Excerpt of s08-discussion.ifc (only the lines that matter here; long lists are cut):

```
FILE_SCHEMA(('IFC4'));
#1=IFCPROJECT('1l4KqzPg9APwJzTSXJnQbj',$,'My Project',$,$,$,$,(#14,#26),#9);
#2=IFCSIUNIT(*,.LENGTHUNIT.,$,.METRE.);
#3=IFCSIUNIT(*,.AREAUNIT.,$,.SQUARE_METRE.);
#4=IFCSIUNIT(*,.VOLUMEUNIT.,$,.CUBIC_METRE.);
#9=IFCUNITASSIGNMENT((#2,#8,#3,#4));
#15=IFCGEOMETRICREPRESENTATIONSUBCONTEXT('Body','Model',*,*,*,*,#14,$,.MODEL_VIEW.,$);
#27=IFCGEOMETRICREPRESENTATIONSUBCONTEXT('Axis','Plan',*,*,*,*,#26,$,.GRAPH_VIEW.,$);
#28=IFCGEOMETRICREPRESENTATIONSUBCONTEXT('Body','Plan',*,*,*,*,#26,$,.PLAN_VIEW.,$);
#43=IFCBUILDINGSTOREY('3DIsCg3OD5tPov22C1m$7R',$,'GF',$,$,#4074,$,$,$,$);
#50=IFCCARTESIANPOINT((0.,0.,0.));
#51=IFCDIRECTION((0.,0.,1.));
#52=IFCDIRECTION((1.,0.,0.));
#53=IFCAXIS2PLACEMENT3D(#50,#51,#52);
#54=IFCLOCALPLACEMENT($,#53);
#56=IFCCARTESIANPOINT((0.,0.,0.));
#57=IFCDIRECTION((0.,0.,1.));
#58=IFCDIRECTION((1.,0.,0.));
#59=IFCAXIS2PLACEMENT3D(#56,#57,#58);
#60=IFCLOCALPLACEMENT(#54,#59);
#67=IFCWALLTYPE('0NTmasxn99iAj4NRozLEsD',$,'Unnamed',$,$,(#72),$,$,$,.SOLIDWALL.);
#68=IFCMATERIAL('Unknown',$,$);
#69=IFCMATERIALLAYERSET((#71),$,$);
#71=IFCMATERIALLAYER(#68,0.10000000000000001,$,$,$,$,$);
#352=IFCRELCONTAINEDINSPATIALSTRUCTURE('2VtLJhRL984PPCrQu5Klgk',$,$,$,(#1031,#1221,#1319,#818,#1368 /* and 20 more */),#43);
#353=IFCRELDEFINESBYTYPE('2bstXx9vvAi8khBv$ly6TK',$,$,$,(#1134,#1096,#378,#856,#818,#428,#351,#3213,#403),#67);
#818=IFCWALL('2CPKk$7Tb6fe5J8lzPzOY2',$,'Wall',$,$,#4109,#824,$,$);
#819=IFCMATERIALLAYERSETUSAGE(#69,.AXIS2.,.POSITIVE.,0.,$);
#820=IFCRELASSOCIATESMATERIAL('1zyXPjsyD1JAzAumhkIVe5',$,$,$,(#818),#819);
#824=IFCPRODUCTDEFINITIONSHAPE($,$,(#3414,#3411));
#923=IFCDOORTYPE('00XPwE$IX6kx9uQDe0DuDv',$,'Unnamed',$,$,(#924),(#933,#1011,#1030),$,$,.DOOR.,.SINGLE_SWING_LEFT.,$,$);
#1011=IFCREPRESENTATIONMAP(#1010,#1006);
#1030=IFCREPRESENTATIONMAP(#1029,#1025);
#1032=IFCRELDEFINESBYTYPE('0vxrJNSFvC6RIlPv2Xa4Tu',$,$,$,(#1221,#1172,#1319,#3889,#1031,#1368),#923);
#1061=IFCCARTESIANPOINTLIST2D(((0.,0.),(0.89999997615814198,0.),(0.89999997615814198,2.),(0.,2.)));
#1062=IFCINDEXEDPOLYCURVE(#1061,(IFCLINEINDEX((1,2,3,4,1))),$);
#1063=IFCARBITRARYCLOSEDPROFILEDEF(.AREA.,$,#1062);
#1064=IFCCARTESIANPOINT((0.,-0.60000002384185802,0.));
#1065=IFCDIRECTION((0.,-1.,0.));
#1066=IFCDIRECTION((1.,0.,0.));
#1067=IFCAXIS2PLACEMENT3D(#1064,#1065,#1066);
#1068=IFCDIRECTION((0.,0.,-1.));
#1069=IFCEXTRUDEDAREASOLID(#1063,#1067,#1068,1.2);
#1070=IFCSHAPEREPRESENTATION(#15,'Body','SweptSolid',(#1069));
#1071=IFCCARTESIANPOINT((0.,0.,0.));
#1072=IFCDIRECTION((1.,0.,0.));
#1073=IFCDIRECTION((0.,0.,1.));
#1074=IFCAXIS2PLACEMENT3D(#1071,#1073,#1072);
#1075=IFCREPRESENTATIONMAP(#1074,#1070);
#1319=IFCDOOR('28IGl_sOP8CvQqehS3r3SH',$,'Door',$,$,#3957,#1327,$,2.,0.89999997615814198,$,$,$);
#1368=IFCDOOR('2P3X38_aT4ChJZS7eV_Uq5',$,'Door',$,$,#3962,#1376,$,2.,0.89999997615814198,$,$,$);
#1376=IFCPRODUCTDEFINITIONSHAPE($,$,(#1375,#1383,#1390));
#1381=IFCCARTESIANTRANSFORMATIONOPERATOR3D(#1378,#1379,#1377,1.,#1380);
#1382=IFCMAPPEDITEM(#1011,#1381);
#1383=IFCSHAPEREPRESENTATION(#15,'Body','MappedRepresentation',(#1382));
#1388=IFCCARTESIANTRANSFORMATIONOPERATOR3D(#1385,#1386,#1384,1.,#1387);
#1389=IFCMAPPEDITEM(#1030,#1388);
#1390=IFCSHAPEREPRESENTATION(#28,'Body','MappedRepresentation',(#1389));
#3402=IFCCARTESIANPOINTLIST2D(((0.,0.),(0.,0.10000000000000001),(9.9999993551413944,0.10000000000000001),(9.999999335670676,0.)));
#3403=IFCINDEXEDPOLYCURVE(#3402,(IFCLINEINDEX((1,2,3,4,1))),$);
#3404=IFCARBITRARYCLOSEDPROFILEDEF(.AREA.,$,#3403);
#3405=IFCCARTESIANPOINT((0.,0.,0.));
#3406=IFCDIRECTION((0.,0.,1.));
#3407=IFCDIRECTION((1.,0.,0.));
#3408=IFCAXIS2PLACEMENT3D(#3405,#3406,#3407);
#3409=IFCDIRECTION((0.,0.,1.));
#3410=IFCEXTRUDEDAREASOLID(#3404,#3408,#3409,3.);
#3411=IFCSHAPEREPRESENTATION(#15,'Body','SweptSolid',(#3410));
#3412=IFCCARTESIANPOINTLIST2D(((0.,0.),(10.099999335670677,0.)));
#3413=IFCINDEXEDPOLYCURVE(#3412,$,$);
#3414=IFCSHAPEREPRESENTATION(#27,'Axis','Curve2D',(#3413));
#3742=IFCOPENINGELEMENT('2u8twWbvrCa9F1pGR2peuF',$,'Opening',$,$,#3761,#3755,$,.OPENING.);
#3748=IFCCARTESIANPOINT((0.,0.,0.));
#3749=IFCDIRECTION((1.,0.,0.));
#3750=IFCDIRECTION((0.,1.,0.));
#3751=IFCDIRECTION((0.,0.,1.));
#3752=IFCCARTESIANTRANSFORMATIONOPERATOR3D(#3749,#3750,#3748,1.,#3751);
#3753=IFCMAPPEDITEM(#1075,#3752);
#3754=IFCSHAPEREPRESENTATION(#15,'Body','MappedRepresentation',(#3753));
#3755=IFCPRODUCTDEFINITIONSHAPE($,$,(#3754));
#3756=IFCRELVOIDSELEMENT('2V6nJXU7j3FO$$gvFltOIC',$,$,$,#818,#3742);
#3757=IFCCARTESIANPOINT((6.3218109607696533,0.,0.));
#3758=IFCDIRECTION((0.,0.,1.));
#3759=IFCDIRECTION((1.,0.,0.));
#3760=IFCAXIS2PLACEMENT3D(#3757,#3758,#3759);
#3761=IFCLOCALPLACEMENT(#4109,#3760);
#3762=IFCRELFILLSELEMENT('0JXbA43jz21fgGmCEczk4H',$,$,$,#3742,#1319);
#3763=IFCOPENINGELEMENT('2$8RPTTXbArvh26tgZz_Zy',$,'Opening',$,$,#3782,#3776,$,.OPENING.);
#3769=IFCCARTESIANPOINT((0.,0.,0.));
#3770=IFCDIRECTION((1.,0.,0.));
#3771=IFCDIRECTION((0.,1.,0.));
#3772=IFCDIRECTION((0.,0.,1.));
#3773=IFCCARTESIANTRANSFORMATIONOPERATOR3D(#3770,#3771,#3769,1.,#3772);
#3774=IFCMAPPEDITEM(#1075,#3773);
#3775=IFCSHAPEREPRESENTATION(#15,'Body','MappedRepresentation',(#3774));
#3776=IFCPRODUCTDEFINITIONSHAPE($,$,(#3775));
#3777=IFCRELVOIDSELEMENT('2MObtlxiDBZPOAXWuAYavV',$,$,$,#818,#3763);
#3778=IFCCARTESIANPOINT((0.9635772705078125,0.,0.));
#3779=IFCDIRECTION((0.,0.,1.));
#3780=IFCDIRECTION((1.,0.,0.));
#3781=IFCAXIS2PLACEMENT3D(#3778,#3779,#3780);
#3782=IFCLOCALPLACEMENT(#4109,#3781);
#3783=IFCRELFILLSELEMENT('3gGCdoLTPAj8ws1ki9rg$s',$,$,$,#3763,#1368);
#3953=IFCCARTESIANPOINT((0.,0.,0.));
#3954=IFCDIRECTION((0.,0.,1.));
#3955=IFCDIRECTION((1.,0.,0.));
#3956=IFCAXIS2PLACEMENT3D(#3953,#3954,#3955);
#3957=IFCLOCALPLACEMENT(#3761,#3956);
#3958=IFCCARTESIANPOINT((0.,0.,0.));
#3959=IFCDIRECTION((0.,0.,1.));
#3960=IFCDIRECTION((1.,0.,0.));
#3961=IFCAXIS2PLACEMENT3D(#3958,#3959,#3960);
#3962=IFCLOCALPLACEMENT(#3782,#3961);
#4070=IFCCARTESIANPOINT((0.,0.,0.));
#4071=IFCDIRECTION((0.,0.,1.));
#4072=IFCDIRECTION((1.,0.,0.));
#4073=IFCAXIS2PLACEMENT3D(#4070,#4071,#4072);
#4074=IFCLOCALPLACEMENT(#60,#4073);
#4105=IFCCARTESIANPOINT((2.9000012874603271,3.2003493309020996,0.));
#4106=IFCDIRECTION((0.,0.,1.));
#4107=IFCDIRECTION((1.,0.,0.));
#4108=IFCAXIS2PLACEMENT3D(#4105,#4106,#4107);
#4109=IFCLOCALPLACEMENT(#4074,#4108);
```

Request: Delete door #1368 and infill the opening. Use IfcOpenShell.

```python
import ifcopenshell
import ifcopenshell.api.feature
import ifcopenshell.api.root
import ifcopenshell.geom
import ifcopenshell.util.shape

model = ifcopenshell.open("s08-discussion.ifc")
settings = ifcopenshell.geom.settings()


def volume(element):
    """Net volume in cubic metres, openings subtracted."""
    shape = ifcopenshell.geom.create_shape(settings, element)
    return ifcopenshell.util.shape.get_volume(shape.geometry)


door = model.by_guid("2P3X38_aT4ChJZS7eV_Uq5")
opening = door.FillsVoids[0].RelatingOpeningElement
wall = opening.VoidsElements[0].RelatingBuildingElement
before = volume(wall)

ifcopenshell.api.root.remove_product(model, product=door)
ifcopenshell.api.feature.remove_feature(model, feature=opening)

after = volume(wall)

print(f"wall volume {before:.3f} -> {after:.3f} m3")

model.write("s08-discussion_updated.ifc")
```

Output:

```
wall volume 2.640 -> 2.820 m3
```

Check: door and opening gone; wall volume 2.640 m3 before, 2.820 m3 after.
